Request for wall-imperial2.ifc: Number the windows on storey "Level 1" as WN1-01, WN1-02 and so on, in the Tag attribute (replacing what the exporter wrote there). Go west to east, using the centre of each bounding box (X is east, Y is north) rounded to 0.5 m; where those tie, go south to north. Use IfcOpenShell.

First a look at what the model holds.

```python
import ifcopenshell
import ifcopenshell.util.element
import ifcopenshell.util.placement

model = ifcopenshell.open("wall-imperial2.ifc")
print(model.schema)
storey = next(s for s in model.by_type("IfcBuildingStorey") if s.Name == "Level 1")
windows = [e for e in ifcopenshell.util.element.get_decomposition(storey) if e.is_a("IfcWindow")]
for e in sorted(windows, key=lambda e: e.id()):
    origin = ifcopenshell.util.placement.get_local_placement(e.ObjectPlacement)[:3, 3]
    print(e.id(), e.Tag, e.Name, origin.round(2) + 0.0, sep=" | ")
```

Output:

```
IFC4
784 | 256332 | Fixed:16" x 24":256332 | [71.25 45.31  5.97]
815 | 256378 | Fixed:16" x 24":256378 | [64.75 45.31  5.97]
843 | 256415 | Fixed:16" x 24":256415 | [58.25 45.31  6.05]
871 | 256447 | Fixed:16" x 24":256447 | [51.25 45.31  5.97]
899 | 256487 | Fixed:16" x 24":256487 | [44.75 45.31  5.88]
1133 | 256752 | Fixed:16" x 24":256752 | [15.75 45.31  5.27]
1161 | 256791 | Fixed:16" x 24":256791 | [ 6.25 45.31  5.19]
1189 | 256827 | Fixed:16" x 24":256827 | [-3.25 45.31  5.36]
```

```python
import ifcopenshell
import ifcopenshell.geom
import ifcopenshell.util.element
import ifcopenshell.util.shape

model = ifcopenshell.open("wall-imperial2.ifc")
settings = ifcopenshell.geom.settings()
settings.set("use-world-coords", True)


def centre(element):
    shape = ifcopenshell.geom.create_shape(settings, element)
    return ifcopenshell.util.shape.get_bbox_centroid(shape.geometry)


storey = next(s for s in model.by_type("IfcBuildingStorey") if s.Name == "Level 1")
windows = [e for e in ifcopenshell.util.element.get_decomposition(storey) if e.is_a("IfcWindow")]

# Insertion points can sit at a corner or the storey origin, so sort by the geometry (in metres).
centres = {e: centre(e) for e in windows}
windows.sort(key=lambda e: (round(centres[e][0] / 0.5), centres[e][1]))

for i, e in enumerate(windows, start=1):
    number = f"WN1-{i:02d}"
    e.Tag = number
    print(e.id(), number)

model.write("wall-imperial2_updated.ifc")
```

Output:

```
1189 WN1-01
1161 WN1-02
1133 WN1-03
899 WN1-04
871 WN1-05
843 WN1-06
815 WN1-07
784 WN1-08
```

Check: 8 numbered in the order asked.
